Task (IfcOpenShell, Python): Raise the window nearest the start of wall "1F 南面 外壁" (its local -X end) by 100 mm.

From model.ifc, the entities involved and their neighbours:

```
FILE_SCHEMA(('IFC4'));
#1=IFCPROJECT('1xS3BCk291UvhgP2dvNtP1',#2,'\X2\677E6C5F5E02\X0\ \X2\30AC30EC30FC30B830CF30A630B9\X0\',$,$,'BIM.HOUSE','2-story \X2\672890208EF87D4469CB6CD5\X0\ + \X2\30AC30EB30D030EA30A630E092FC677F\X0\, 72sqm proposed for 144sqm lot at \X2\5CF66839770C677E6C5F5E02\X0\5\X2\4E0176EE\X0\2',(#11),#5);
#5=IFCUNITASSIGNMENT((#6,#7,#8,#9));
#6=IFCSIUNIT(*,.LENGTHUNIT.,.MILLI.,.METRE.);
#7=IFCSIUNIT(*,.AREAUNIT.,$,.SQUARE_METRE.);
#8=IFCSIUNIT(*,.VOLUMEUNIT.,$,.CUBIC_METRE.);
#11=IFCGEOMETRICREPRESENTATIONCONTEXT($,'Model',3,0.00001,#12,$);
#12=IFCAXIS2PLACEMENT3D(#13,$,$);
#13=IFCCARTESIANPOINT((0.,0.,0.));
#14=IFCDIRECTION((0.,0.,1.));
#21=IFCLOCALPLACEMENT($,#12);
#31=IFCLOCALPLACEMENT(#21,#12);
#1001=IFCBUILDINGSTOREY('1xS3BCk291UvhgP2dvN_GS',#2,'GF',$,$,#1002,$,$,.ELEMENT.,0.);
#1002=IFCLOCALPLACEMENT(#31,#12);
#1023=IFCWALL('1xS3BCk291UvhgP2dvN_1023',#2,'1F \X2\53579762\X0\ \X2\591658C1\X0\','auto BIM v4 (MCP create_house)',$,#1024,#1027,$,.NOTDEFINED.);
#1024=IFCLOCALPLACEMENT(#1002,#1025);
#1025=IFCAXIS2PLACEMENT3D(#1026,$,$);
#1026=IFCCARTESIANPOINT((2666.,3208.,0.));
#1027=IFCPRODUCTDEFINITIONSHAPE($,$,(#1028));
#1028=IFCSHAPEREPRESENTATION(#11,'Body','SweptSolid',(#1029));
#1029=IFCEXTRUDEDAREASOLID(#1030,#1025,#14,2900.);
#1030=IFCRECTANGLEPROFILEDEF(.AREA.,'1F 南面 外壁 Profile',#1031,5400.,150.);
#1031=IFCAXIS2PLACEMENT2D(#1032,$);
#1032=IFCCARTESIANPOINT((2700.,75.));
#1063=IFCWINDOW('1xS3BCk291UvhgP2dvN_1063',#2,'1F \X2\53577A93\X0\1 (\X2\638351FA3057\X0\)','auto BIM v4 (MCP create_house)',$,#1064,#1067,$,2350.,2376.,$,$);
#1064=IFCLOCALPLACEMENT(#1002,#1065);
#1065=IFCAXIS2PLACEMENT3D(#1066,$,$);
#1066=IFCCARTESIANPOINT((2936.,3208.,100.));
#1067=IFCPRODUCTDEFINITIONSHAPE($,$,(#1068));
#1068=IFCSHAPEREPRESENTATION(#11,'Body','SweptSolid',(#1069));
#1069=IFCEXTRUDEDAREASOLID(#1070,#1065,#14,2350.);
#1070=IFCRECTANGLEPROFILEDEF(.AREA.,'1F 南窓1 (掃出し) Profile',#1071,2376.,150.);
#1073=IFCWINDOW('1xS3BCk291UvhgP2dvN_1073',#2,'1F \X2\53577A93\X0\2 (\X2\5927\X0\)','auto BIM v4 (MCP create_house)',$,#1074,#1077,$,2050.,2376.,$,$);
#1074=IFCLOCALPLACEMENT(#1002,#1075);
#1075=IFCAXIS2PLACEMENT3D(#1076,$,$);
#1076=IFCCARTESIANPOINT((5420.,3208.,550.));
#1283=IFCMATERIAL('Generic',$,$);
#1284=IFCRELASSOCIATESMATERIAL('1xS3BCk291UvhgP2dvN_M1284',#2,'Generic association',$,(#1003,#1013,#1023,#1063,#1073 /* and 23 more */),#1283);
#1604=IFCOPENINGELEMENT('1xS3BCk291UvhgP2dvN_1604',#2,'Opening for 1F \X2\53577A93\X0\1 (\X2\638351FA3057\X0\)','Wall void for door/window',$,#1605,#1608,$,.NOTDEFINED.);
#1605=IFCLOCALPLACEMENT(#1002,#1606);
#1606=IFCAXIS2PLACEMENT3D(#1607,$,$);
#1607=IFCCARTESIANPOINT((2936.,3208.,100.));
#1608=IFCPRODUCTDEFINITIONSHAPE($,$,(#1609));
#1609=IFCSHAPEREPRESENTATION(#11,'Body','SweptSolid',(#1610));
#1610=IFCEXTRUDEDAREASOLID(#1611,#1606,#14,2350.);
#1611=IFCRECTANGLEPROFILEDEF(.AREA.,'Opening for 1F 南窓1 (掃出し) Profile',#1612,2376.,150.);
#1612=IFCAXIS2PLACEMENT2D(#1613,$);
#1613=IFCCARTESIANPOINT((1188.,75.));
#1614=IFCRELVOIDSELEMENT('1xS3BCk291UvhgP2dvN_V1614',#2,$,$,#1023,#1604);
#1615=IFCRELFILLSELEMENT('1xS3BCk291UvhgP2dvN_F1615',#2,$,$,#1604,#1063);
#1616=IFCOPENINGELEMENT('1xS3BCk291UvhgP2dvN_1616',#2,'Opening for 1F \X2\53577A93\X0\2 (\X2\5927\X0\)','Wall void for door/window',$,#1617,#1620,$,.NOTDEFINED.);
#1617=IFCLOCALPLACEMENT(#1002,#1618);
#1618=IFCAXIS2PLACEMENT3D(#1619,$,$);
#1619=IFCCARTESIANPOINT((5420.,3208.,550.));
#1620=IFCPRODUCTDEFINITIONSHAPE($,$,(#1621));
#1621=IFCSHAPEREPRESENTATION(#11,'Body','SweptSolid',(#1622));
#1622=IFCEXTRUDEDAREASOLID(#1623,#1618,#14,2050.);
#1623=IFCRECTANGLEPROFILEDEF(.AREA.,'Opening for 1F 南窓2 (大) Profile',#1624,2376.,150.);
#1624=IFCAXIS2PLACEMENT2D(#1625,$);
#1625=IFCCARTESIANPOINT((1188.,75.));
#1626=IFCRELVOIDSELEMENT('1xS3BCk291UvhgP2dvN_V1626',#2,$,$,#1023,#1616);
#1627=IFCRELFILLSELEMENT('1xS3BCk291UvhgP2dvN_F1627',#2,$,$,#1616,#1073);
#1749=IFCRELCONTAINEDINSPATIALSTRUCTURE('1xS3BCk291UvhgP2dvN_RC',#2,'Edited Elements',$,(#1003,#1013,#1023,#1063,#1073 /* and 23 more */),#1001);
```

```python
import numpy as np
import ifcopenshell
import ifcopenshell.api.geometry
import ifcopenshell.util.placement
import ifcopenshell.util.unit

model = ifcopenshell.open("model.ifc")
unit_scale = ifcopenshell.util.unit.calculate_unit_scale(model)

window = model.by_guid("1xS3BCk291UvhgP2dvN_1063")
opening = window.FillsVoids[0].RelatingOpeningElement
dz = 100.0

shift = np.array([0.0, 0.0, dz])
# The window is not placed relative to its opening, so move both.
for product in (opening, window):
    matrix = ifcopenshell.util.placement.get_local_placement(product.ObjectPlacement)
    matrix[:3, 3] += shift
    ifcopenshell.api.geometry.edit_object_placement(model, product=product, matrix=matrix, is_si=False)

print(f"moved by {dz * unit_scale:+.3f} m")

model.write("model_edited.ifc")
```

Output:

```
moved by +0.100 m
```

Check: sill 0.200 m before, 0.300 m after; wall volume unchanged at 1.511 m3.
